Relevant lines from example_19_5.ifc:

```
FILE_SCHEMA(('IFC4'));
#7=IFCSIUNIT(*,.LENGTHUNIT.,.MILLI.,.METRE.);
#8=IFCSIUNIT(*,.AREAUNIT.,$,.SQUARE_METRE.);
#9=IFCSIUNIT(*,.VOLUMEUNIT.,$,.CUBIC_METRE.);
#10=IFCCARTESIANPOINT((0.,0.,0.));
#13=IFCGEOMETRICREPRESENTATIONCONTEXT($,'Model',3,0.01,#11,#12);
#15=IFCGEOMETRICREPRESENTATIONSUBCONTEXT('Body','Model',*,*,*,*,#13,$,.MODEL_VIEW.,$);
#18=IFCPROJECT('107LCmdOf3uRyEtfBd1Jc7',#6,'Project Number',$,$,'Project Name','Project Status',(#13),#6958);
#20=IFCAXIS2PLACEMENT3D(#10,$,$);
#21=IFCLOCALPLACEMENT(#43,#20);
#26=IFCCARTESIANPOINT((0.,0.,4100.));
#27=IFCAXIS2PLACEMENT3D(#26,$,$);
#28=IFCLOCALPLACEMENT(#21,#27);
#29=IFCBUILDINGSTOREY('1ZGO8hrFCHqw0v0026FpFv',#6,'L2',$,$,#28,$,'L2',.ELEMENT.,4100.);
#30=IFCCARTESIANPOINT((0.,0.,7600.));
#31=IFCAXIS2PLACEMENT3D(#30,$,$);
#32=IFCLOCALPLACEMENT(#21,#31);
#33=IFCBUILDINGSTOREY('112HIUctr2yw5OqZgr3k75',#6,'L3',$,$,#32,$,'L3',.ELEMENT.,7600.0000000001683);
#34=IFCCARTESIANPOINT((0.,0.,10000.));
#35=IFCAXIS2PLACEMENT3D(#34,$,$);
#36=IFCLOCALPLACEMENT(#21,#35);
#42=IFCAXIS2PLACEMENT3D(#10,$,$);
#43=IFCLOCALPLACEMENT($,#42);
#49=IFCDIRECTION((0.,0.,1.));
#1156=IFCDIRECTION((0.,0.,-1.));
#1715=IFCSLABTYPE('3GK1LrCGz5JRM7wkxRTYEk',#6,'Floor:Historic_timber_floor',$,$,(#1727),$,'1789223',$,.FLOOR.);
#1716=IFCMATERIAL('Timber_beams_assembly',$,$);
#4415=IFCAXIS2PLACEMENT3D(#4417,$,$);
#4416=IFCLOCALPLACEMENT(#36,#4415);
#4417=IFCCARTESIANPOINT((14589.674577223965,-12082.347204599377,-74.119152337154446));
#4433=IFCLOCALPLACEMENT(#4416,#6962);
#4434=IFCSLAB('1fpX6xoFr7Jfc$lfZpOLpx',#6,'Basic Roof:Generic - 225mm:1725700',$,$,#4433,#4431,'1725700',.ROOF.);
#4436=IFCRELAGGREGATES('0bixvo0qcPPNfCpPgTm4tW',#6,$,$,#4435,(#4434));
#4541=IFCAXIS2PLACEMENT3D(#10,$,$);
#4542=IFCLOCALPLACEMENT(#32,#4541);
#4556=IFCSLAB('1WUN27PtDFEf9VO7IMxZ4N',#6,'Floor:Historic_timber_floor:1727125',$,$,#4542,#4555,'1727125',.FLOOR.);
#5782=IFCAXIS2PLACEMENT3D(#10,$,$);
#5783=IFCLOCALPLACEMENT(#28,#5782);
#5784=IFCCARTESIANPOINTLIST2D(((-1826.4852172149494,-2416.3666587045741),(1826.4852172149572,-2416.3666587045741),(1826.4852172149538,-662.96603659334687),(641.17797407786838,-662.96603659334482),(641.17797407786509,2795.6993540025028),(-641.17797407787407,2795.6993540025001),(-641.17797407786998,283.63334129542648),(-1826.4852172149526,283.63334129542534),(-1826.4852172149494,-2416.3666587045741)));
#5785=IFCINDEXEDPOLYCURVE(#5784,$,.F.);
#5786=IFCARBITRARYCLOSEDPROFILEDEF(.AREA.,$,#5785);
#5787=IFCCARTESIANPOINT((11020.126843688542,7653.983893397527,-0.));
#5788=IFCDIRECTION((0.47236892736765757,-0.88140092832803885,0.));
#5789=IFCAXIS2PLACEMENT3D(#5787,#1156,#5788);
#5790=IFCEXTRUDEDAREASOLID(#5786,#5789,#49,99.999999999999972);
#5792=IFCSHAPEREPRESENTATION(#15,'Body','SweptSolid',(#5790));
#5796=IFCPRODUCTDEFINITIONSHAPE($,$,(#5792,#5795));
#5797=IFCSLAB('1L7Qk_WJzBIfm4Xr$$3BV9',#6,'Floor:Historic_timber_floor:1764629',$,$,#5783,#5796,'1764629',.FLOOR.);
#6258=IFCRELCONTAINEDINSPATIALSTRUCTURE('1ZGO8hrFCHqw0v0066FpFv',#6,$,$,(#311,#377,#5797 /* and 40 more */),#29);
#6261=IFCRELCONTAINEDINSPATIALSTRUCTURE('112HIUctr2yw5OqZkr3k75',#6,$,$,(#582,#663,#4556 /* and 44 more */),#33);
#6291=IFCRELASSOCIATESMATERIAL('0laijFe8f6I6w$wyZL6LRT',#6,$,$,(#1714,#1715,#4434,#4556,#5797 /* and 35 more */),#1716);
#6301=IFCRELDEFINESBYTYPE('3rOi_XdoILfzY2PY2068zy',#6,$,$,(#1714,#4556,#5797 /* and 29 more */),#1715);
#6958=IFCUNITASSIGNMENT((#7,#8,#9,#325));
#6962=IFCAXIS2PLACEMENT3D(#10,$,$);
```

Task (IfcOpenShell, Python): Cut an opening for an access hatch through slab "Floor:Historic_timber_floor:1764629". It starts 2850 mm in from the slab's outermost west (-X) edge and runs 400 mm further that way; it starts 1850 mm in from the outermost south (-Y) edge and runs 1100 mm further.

```python
import numpy as np
import ifcopenshell
import ifcopenshell.api.feature
import ifcopenshell.api.geometry
import ifcopenshell.api.root
import ifcopenshell.geom
import ifcopenshell.util.placement
import ifcopenshell.util.representation
import ifcopenshell.util.shape
import ifcopenshell.util.unit

model = ifcopenshell.open("example_19_5.ifc")
unit_scale = ifcopenshell.util.unit.calculate_unit_scale(model)
settings = ifcopenshell.geom.settings()


def volume(element):
    """Net volume in cubic metres, openings subtracted."""
    shape = ifcopenshell.geom.create_shape(settings, element)
    return ifcopenshell.util.shape.get_volume(shape.geometry)


slab = model.by_id(5797)
before = volume(slab)

# Extent in the slab's own axes, in metres. The edges named are its -X and -Y sides.
slab_shape = ifcopenshell.geom.create_shape(settings, slab)
vertices = ifcopenshell.util.shape.get_vertices(slab_shape.geometry)
x_min, y_min, bottom = vertices.min(axis=0)
top = vertices[:, 2].max()

opening = ifcopenshell.api.root.create_entity(model, ifc_class="IfcOpeningElement", name="Access hatch opening", predefined_type="OPENING")
context = ifcopenshell.util.representation.get_context(model, "Model", "Body", "MODEL_VIEW")
width, depth = 0.4, 1.1
outline = [(0.0, 0.0), (width, 0.0), (width, depth), (0.0, depth), (0.0, 0.0)]
# Overshoot both faces by 50 mm so the cut is clean.
shape = ifcopenshell.api.geometry.add_slab_representation(
    model, context=context, depth=top - bottom + 0.1, polyline=outline
)
ifcopenshell.api.geometry.assign_representation(model, product=opening, representation=shape)

matrix = ifcopenshell.util.placement.get_local_placement(slab.ObjectPlacement)
matrix[:, 3] = matrix @ np.append(np.array([x_min + 2.85, y_min + 1.85, bottom - 0.05]) / unit_scale, 1.0)
ifcopenshell.api.geometry.edit_object_placement(model, product=opening, matrix=matrix, is_si=False)
ifcopenshell.api.feature.add_feature(model, feature=opening, element=slab)

after = volume(slab)

print(f"slab volume {before:.3f} -> {after:.3f} m3")

model.write("example_19_5_updated.ifc")
```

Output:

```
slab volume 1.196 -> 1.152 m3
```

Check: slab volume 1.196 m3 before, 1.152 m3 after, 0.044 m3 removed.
